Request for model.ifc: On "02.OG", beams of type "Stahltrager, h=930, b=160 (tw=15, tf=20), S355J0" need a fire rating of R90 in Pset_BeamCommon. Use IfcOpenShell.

First a look at what the model holds.

```python
import ifcopenshell
import ifcopenshell.util.element

model = ifcopenshell.open("model.ifc")
print(model.schema)
storey = next(s for s in model.by_type("IfcBuildingStorey") if s.Name == "02.OG")
beams = [e for e in ifcopenshell.util.element.get_decomposition(storey) if e.is_a("IfcBeam")]
seen = {}
for e in beams:
    element_type = ifcopenshell.util.element.get_type(e)
    key = (element_type.Name if element_type != e and element_type else None, ifcopenshell.util.element.get_pset(e, "Pset_BeamCommon", "FireRating"))
    seen[key] = seen.get(key, 0) + 1
for (name, value), count in sorted(seen.items(), key=str):
    print(count, "x", name, "|", value)
```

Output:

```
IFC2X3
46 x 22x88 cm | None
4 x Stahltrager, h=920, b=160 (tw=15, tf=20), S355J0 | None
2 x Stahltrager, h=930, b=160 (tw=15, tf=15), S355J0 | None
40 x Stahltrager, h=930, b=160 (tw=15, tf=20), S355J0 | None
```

```python
import ifcopenshell
import ifcopenshell.api.pset
import ifcopenshell.util.element

model = ifcopenshell.open("model.ifc")

storey = next(s for s in model.by_type("IfcBuildingStorey") if s.Name == "02.OG")
beams = [e for e in ifcopenshell.util.element.get_decomposition(storey) if e.is_a("IfcBeam")]

count = 0
for e in beams:
    element_type = ifcopenshell.util.element.get_type(e)
    if element_type in (None, e) or element_type.Name != "Stahltrager, h=930, b=160 (tw=15, tf=20), S355J0":
        continue
    # add_pset returns the element's existing set when there is one.
    pset = ifcopenshell.api.pset.add_pset(model, product=e, name="Pset_BeamCommon")
    ifcopenshell.api.pset.edit_pset(model, pset=pset, properties={"FireRating": "R90"})
    count += 1

print(count, "beams updated")

model.write("model_v2.ifc")
```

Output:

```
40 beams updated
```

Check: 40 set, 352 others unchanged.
